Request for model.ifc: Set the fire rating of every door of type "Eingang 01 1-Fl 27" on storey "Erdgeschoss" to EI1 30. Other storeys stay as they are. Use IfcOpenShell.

First a look at what the model holds.

```python
import ifcopenshell
import ifcopenshell.util.element

model = ifcopenshell.open("model.ifc")
print(model.schema)
storey = next(s for s in model.by_type("IfcBuildingStorey") if s.Name == "Erdgeschoss")
doors = [e for e in ifcopenshell.util.element.get_decomposition(storey) if e.is_a("IfcDoor")]
seen = {}
for e in doors:
    element_type = ifcopenshell.util.element.get_type(e)
    key = (element_type.Name if element_type != e and element_type else None, ifcopenshell.util.element.get_pset(e, "Pset_DoorCommon", "FireRating"))
    seen[key] = seen.get(key, 0) + 1
for (name, value), count in sorted(seen.items(), key=str):
    print(count, "x", name, "|", value)
```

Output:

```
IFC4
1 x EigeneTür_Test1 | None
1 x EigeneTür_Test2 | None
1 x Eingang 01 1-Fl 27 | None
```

```python
import ifcopenshell
import ifcopenshell.api.pset
import ifcopenshell.util.element

model = ifcopenshell.open("model.ifc")

storey = next(s for s in model.by_type("IfcBuildingStorey") if s.Name == "Erdgeschoss")
doors = [e for e in ifcopenshell.util.element.get_decomposition(storey) if e.is_a("IfcDoor")]

count = 0
for e in doors:
    element_type = ifcopenshell.util.element.get_type(e)
    if element_type in (None, e) or element_type.Name != "Eingang 01 1-Fl 27":
        continue
    # add_pset returns the element's existing set when there is one.
    pset = ifcopenshell.api.pset.add_pset(model, product=e, name="Pset_DoorCommon")
    ifcopenshell.api.pset.edit_pset(model, pset=pset, properties={"FireRating": "EI1 30"})
    count += 1

print(count, "doors updated")

model.write("model-out.ifc")
```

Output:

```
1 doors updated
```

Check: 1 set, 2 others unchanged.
